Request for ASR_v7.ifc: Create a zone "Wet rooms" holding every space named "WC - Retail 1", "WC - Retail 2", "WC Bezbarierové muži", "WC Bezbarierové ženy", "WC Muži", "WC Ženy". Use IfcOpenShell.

First a look at what the model holds.

```python
import ifcopenshell

model = ifcopenshell.open("ASR_v7.ifc")
print(model.schema)
seen = {}
for space in model.by_type("IfcSpace"):
    seen[space.LongName] = seen.get(space.LongName, 0) + 1
for name, count in sorted(seen.items(), key=str):
    print(count, "x", name)
print("zones:", [z.Name for z in model.by_type("IfcZone")][:20])
```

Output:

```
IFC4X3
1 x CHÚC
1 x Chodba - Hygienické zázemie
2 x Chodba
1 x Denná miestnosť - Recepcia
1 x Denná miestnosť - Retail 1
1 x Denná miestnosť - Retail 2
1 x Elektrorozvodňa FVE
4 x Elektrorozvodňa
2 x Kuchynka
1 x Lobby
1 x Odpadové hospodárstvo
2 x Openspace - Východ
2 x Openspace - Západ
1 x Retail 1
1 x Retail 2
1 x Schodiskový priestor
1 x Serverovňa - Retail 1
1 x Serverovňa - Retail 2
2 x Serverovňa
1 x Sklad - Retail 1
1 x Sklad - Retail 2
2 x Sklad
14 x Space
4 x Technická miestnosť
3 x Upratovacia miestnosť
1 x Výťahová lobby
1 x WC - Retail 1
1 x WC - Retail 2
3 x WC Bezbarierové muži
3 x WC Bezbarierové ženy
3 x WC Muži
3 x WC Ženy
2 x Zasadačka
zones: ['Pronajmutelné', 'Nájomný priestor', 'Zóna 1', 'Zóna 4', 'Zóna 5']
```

```python
import ifcopenshell
import ifcopenshell.api.group
import ifcopenshell.api.root

model = ifcopenshell.open("ASR_v7.ifc")

names = {"WC - Retail 1", "WC - Retail 2", "WC Bezbarierové muži", "WC Bezbarierové ženy", "WC Muži", "WC Ženy"}
spaces = [s for s in model.by_type("IfcSpace") if s.LongName in names]

zone = ifcopenshell.api.root.create_entity(model, ifc_class="IfcZone", name="Wet rooms")
ifcopenshell.api.group.assign_group(model, products=spaces, group=zone)
print(len(spaces), "spaces in", zone.Name)

model.write("ASR_v7_edited.ifc")
```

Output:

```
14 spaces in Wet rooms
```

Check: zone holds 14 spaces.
